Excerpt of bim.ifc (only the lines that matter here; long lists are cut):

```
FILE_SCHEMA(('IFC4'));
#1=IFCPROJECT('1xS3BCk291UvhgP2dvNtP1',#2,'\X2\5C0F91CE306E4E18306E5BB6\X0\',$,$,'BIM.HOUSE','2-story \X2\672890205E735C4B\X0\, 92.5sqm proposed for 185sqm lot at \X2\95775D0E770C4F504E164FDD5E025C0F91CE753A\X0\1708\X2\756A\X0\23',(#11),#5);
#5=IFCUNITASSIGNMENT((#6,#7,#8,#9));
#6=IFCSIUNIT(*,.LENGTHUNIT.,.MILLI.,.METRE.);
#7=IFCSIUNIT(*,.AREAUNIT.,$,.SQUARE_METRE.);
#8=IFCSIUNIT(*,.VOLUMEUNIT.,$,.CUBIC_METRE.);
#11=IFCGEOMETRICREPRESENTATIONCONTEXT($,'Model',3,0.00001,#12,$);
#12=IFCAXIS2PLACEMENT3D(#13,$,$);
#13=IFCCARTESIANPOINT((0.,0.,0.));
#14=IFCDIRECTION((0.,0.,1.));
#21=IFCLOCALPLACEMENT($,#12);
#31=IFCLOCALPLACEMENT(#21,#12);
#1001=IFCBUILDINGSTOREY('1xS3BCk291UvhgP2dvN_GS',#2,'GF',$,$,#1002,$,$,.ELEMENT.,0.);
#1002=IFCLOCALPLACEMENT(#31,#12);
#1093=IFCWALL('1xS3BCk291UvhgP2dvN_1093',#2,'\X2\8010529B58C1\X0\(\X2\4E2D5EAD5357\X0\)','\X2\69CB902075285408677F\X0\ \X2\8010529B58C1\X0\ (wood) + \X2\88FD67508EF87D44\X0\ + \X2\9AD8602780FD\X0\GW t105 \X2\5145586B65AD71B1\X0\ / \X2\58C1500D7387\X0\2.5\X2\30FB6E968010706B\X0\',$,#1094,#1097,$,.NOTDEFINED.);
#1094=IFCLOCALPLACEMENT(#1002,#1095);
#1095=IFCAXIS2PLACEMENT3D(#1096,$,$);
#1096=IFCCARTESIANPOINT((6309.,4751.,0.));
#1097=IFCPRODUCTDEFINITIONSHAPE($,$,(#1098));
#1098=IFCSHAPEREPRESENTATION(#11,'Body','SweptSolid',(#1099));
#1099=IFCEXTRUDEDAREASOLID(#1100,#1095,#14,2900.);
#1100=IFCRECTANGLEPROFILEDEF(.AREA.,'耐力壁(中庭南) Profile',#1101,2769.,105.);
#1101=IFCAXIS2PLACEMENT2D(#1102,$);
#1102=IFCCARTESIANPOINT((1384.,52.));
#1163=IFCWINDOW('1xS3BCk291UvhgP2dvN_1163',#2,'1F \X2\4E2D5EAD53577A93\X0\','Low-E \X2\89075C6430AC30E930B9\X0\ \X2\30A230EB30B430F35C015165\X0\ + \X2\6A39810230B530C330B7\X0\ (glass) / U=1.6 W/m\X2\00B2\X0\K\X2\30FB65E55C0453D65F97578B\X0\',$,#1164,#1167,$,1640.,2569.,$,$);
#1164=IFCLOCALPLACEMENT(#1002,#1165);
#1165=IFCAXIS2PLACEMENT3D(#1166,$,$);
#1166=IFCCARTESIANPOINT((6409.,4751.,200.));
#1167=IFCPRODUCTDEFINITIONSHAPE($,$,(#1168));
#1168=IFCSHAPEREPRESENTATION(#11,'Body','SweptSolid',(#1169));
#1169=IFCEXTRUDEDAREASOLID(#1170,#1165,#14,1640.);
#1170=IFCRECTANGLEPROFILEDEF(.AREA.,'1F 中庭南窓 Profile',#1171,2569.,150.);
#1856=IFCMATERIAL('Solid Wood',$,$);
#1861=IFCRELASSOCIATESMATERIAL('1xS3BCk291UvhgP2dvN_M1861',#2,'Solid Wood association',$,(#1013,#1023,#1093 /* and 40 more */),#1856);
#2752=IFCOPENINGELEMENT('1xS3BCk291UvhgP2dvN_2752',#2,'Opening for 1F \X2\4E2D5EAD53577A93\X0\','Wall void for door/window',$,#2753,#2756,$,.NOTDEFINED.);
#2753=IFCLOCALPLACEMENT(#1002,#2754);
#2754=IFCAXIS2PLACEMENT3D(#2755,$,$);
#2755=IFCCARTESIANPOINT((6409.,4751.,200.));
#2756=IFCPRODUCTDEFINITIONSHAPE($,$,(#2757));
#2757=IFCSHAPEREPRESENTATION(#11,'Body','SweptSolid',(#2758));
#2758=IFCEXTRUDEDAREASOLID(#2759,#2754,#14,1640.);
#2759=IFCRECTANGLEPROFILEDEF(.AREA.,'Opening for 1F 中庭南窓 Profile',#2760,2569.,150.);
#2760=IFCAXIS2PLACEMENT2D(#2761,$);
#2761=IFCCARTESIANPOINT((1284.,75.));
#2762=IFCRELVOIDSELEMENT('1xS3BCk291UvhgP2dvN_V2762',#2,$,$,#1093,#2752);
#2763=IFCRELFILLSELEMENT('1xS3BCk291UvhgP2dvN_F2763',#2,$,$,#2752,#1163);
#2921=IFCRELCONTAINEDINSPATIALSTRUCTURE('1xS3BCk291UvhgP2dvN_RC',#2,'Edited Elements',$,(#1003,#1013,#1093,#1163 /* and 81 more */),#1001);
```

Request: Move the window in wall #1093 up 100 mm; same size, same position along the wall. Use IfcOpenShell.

```python
import numpy as np
import ifcopenshell
import ifcopenshell.api.geometry
import ifcopenshell.util.placement
import ifcopenshell.util.unit

model = ifcopenshell.open("bim.ifc")
unit_scale = ifcopenshell.util.unit.calculate_unit_scale(model)

window = model.by_id(1163)
opening = window.FillsVoids[0].RelatingOpeningElement
dz = 100.0

shift = np.array([0.0, 0.0, dz])
# The window is not placed relative to its opening, so move both.
for product in (opening, window):
    matrix = ifcopenshell.util.placement.get_local_placement(product.ObjectPlacement)
    matrix[:3, 3] += shift
    ifcopenshell.api.geometry.edit_object_placement(model, product=product, matrix=matrix, is_si=False)

print(f"moved by {dz * unit_scale:+.3f} m")

model.write("bim_edited.ifc")
```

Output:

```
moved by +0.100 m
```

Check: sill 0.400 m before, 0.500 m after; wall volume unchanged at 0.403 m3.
